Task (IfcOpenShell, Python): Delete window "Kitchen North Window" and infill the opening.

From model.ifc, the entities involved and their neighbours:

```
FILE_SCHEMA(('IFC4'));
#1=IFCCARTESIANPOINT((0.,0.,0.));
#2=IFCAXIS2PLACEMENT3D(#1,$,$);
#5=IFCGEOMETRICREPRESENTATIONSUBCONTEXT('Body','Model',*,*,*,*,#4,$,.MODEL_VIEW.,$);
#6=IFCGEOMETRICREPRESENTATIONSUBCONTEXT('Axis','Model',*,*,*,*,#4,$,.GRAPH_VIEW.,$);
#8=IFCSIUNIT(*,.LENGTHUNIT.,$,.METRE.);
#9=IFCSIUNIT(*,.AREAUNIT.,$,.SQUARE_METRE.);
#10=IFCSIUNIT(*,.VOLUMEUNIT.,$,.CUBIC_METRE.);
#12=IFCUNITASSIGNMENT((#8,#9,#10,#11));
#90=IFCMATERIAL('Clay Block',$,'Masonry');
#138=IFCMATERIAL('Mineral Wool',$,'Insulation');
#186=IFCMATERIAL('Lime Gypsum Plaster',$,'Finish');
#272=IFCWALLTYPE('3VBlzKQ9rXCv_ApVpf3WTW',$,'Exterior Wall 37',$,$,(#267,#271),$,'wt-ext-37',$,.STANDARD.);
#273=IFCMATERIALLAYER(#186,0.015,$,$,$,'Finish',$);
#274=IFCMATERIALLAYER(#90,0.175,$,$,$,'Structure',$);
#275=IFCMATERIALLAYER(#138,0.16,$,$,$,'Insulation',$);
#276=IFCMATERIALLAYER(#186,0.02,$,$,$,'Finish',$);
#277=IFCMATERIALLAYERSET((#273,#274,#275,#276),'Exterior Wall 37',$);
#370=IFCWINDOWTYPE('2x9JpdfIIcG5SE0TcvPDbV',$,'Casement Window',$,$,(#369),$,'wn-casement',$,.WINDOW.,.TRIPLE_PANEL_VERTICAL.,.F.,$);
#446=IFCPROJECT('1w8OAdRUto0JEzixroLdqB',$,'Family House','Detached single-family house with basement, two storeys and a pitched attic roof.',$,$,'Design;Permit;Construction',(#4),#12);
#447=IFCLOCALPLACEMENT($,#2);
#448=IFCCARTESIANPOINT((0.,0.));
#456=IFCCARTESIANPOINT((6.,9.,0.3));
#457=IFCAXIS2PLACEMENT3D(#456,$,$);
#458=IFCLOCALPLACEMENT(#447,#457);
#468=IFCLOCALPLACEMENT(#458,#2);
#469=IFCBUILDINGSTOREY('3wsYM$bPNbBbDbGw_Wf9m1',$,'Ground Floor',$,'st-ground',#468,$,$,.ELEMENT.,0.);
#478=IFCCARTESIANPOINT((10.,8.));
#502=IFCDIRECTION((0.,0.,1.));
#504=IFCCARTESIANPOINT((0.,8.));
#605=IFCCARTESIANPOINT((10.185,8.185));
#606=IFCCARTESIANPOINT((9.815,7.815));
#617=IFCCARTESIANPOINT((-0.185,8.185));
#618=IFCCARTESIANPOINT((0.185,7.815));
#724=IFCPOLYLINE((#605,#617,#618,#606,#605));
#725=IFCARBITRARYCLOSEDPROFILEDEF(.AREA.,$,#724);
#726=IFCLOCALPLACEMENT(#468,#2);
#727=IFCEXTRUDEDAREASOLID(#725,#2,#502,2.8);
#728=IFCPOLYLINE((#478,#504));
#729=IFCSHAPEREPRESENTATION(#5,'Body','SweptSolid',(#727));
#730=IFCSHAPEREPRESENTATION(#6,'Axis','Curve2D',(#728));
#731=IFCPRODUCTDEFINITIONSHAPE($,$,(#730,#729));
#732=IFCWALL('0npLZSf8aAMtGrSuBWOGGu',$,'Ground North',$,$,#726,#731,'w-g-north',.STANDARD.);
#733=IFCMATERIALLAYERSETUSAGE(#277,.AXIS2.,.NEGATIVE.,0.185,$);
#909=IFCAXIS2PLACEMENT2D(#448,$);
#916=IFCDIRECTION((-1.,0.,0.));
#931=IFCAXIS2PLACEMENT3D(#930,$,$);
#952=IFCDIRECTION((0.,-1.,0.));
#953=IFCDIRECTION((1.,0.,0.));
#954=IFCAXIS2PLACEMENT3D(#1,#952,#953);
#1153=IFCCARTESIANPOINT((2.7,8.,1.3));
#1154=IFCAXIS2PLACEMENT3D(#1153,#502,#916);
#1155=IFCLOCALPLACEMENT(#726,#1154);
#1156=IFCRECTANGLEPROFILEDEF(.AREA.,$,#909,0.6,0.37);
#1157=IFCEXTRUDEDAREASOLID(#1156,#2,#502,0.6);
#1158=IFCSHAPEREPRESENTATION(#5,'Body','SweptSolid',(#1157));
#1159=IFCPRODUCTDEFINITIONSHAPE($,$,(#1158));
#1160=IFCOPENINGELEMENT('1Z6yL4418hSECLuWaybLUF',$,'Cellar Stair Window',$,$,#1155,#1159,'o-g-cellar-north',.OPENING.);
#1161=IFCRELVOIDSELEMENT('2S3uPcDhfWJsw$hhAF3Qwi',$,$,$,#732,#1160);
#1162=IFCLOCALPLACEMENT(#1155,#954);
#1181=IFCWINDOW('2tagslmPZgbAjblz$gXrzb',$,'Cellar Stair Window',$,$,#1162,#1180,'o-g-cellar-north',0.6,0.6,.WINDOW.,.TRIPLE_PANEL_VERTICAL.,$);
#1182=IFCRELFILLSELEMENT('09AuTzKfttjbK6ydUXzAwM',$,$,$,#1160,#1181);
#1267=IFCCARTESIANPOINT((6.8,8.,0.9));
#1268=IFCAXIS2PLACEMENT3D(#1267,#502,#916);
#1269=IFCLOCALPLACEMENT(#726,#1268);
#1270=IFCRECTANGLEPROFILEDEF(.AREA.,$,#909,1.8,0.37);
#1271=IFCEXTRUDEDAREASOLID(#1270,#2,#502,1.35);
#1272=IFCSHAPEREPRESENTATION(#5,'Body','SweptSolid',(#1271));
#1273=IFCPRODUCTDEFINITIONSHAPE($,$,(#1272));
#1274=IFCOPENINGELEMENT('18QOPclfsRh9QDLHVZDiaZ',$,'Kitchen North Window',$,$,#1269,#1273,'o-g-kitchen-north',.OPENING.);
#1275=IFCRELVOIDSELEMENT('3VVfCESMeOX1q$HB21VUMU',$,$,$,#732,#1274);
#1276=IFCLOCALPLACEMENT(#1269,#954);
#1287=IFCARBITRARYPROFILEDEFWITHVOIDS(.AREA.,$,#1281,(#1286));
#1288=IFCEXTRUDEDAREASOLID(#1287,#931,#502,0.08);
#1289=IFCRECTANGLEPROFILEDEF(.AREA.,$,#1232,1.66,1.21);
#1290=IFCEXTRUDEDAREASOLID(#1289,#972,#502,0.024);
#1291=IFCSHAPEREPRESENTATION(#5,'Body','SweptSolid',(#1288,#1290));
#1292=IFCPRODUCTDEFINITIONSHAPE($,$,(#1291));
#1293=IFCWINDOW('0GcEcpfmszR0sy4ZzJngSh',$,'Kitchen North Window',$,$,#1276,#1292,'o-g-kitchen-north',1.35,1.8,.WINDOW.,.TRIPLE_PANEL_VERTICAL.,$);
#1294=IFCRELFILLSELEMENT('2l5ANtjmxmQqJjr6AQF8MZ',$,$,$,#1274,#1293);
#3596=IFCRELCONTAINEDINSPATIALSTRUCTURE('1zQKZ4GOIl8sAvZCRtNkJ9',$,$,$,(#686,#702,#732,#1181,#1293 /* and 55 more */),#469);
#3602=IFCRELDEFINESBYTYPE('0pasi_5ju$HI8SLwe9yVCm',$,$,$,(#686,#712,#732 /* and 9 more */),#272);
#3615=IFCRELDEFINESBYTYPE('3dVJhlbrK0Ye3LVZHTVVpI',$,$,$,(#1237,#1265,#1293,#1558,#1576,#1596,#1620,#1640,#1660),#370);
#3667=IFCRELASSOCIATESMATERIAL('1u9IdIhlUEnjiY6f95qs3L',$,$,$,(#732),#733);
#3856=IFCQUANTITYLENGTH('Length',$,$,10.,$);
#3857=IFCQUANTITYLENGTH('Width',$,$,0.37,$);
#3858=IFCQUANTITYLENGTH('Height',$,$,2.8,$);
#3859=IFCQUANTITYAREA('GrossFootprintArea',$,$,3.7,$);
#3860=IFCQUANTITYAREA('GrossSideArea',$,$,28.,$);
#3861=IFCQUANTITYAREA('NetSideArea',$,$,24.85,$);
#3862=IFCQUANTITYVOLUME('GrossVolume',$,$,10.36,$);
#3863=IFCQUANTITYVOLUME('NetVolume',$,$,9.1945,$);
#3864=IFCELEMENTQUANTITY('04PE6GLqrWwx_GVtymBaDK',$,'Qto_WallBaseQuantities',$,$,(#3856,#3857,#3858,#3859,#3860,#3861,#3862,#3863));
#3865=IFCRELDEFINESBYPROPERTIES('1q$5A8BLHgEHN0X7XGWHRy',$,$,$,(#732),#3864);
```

```python
import ifcopenshell
import ifcopenshell.api.feature
import ifcopenshell.api.pset
import ifcopenshell.api.root
import ifcopenshell.geom
import ifcopenshell.util.element
import ifcopenshell.util.shape
import ifcopenshell.util.unit

model = ifcopenshell.open("model.ifc")
area_scale = ifcopenshell.util.unit.calculate_unit_scale(model, "AREAUNIT")
volume_scale = ifcopenshell.util.unit.calculate_unit_scale(model, "VOLUMEUNIT")
settings = ifcopenshell.geom.settings()


def volume(element):
    """Net volume in cubic metres, openings subtracted."""
    shape = ifcopenshell.geom.create_shape(settings, element)
    return ifcopenshell.util.shape.get_volume(shape.geometry)


window = model.by_id(1293)
opening = window.FillsVoids[0].RelatingOpeningElement
wall = opening.VoidsElements[0].RelatingBuildingElement
before = volume(wall)

ifcopenshell.api.root.remove_product(model, product=window)
ifcopenshell.api.feature.remove_feature(model, feature=opening)

after = volume(wall)
thickness = 0.37  # wall thickness in metres

# Update the wall's stored quantities.
qto = model.by_id(ifcopenshell.util.element.get_pset(wall, "Qto_WallBaseQuantities", should_inherit=False)["id"])
ifcopenshell.api.pset.edit_qto(model, qto=qto, properties={
    "NetSideArea": after / thickness / area_scale,
    "NetVolume": after / volume_scale,
})

print(f"wall volume {before:.3f} -> {after:.3f} m3")

model.write("model-out.ifc")
```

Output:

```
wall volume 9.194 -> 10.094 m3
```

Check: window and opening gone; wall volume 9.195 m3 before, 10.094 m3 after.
